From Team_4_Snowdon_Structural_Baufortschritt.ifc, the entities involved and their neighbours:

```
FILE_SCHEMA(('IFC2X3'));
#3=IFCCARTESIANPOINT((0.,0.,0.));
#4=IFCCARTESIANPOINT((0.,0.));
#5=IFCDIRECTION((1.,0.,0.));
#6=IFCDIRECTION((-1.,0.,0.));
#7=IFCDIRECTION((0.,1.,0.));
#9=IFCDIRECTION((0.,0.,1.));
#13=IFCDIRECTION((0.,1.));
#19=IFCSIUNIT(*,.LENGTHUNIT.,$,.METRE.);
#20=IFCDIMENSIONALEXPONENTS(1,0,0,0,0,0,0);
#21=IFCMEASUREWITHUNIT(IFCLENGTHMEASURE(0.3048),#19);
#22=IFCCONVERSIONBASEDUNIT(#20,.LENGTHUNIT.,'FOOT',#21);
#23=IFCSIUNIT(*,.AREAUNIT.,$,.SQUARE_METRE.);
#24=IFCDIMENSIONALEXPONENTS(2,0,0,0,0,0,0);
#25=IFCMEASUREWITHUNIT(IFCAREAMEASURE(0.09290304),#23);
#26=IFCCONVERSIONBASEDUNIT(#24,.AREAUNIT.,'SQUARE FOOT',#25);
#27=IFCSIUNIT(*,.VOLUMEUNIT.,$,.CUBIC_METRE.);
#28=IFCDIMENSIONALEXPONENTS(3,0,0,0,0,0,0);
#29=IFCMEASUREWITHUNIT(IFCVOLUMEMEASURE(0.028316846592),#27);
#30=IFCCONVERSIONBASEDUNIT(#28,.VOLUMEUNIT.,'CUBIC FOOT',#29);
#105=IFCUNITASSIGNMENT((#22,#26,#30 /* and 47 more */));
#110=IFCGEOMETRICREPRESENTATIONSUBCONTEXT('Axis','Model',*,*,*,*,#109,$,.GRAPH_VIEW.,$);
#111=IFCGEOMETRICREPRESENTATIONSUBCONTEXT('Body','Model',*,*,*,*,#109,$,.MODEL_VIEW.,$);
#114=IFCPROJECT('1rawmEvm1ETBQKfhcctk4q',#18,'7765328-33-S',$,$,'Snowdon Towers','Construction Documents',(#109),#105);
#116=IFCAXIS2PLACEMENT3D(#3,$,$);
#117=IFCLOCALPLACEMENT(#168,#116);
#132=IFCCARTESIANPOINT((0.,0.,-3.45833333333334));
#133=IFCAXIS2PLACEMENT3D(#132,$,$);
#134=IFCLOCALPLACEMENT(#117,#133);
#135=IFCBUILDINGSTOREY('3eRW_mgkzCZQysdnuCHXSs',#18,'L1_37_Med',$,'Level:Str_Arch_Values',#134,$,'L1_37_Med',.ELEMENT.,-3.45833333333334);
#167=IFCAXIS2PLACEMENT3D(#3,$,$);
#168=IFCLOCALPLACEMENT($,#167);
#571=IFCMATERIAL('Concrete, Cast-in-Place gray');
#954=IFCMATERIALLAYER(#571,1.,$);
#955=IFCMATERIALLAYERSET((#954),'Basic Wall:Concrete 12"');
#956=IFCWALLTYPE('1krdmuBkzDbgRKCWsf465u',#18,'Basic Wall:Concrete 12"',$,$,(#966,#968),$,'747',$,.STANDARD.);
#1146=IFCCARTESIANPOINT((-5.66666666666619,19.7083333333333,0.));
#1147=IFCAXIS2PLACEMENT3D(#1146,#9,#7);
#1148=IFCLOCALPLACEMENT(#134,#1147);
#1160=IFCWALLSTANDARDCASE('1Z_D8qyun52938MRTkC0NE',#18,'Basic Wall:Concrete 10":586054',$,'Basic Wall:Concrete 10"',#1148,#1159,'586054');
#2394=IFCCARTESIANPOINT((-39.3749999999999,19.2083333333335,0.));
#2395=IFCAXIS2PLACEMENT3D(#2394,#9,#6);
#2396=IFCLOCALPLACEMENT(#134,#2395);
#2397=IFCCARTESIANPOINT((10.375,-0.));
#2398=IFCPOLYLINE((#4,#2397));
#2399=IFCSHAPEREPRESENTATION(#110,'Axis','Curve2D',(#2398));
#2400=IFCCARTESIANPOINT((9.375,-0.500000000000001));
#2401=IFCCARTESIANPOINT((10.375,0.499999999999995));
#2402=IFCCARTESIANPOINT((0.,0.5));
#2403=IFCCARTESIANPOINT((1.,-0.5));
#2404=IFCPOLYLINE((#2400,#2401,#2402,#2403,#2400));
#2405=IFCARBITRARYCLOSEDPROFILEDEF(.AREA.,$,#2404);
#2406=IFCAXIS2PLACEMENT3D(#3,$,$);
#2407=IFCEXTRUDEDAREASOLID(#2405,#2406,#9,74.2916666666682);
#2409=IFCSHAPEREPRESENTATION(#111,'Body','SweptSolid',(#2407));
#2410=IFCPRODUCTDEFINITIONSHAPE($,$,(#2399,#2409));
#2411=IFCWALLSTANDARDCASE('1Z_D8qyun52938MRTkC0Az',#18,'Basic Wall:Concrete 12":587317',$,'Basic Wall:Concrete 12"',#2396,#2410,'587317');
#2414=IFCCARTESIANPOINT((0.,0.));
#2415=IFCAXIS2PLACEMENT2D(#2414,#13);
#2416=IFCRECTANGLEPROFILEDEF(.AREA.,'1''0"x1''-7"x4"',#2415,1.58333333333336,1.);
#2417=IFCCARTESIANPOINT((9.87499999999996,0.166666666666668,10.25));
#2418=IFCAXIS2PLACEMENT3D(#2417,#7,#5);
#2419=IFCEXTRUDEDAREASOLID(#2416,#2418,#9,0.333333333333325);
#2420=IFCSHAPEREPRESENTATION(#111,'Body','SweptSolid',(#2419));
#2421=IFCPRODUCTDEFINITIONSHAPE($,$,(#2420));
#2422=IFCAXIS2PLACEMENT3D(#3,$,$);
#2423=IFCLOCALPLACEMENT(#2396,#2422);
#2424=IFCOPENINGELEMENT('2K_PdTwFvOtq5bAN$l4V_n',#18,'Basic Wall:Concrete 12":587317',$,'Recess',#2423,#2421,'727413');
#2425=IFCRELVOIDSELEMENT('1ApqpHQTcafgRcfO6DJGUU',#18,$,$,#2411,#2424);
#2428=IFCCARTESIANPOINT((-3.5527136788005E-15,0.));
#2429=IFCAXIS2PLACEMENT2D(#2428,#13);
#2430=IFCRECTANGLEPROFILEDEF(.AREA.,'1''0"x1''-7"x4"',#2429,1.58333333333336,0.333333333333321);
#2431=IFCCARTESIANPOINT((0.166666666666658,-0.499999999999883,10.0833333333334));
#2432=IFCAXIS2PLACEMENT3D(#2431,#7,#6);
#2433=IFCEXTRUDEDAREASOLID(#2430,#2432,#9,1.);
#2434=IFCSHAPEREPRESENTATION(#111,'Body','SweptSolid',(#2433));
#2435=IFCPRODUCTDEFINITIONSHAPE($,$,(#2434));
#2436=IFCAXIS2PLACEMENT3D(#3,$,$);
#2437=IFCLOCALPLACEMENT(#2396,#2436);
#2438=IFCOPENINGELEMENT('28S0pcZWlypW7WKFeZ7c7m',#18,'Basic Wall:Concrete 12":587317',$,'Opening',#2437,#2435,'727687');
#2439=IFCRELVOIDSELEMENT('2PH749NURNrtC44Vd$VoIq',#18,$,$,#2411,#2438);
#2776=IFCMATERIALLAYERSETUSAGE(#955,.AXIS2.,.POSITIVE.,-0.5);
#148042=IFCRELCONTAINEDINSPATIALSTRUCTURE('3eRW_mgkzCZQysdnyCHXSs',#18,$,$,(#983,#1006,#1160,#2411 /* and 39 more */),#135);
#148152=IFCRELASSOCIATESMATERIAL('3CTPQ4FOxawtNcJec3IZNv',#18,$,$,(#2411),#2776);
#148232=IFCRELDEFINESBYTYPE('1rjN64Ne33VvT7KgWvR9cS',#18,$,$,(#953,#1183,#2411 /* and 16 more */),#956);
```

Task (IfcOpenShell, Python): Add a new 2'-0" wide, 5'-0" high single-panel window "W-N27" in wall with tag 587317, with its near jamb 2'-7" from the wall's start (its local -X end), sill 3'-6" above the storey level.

```python
import numpy as np
import ifcopenshell
import ifcopenshell.api.feature
import ifcopenshell.api.geometry
import ifcopenshell.api.root
import ifcopenshell.api.spatial
import ifcopenshell.api.type
import ifcopenshell.geom
import ifcopenshell.util.element
import ifcopenshell.util.placement
import ifcopenshell.util.representation
import ifcopenshell.util.shape
import ifcopenshell.util.unit

model = ifcopenshell.open("Team_4_Snowdon_Structural_Baufortschritt.ifc")
unit_scale = ifcopenshell.util.unit.calculate_unit_scale(model)
settings = ifcopenshell.geom.settings()


def volume(element):
    """Net volume in cubic metres, openings subtracted."""
    shape = ifcopenshell.geom.create_shape(settings, element)
    return ifcopenshell.util.shape.get_volume(shape.geometry)


wall = model.by_id(2411)
storey = ifcopenshell.util.element.get_container(wall, ifc_class="IfcBuildingStorey")
context = ifcopenshell.util.representation.get_context(model, "Model", "Body", "MODEL_VIEW")
before = volume(wall)

width, height, from_end, sill = 0.6096, 1.524, 0.7874, 1.0668  # metres

# The wall runs along its own X axis, and the end named is its -X end.
wall_shape = ifcopenshell.geom.create_shape(settings, wall)
x, y, z = ifcopenshell.util.shape.get_vertices(wall_shape.geometry).T
start = x.min() + from_end
face, thickness = float(y.min()), float(y.max() - y.min())
wall_matrix = ifcopenshell.util.placement.get_local_placement(wall.ObjectPlacement)
level = ifcopenshell.util.placement.get_local_placement(storey.ObjectPlacement)[2, 3]


def in_wall(x, y):
    """Placement at x, y metres in the wall's axes, at sill height."""
    matrix = wall_matrix.copy()
    matrix[:, 3] = wall_matrix @ np.array([x / unit_scale, y / unit_scale, 0.0, 1.0])
    matrix[2, 3] = level + sill / unit_scale
    return matrix


# Opening: a box that overshoots both wall faces by 50 mm.
opening = ifcopenshell.api.root.create_entity(model, ifc_class="IfcOpeningElement")
box = ifcopenshell.api.geometry.add_wall_representation(
    model, context=context, length=width, height=height, thickness=thickness + 0.1
)
ifcopenshell.api.geometry.assign_representation(model, product=opening, representation=box)
ifcopenshell.api.geometry.edit_object_placement(model, product=opening, matrix=in_wall(start, face - 0.05), is_si=False)
ifcopenshell.api.feature.add_feature(model, feature=opening, element=wall)

window = ifcopenshell.api.root.create_entity(model, ifc_class="IfcWindow", name="W-N27")
window.OverallWidth, window.OverallHeight = width / unit_scale, height / unit_scale
body = ifcopenshell.api.geometry.add_window_representation(
    model,
    context=context,
    overall_width=window.OverallWidth,
    overall_height=window.OverallHeight,
    partition_type="SINGLE_PANEL",
)
ifcopenshell.api.geometry.assign_representation(model, product=window, representation=body)
ifcopenshell.api.spatial.assign_container(model, products=[window], relating_structure=storey)
fills = ifcopenshell.api.feature.add_filling(model, opening=opening, element=window)
fills.OwnerHistory = window.OwnerHistory  # required in IFC2X3

# IFC2X3 keeps the operation on the window style.
style = ifcopenshell.api.root.create_entity(model, ifc_class="IfcWindowStyle", name="W-N27")
style.OperationType, style.ConstructionType = "SINGLE_PANEL", "NOTDEFINED"
style.ParameterTakesPrecedence = style.Sizeable = False
ifcopenshell.api.type.assign_type(model, related_objects=[window], relating_type=style)

# Centre the window in the wall's thickness.
ifcopenshell.api.geometry.edit_object_placement(model, product=window, matrix=in_wall(start, face), is_si=False)
window_shape = ifcopenshell.geom.create_shape(settings, window)
depth = ifcopenshell.util.shape.get_vertices(window_shape.geometry)[:, 1]
offset = face + thickness / 2 - (depth.min() + depth.max()) / 2
ifcopenshell.api.geometry.edit_object_placement(model, product=window, matrix=in_wall(start, offset), is_si=False)

after = volume(wall)

print(f"wall volume {before:.3f} -> {after:.3f} m3")

model.write("Team_4_Snowdon_Structural_Baufortschritt_updated.ifc")
```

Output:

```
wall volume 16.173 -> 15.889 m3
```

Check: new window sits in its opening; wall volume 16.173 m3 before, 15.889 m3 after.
